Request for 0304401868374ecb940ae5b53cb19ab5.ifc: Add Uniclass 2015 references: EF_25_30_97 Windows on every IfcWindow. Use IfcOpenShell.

First a look at what the model holds.

```python
import ifcopenshell

model = ifcopenshell.open("0304401868374ecb940ae5b53cb19ab5.ifc")
print(model.schema)
print("classifications:", [c.Name for c in model.by_type("IfcClassification")])
for ifc_class in ("IfcDoor", "IfcRoof", "IfcStair", "IfcWall", "IfcWindow"):
    print(ifc_class, len(model.by_type(ifc_class)))
```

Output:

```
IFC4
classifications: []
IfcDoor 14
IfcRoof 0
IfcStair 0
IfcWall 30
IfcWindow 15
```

```python
import ifcopenshell
import ifcopenshell.api.classification

model = ifcopenshell.open("0304401868374ecb940ae5b53cb19ab5.ifc")

system = ifcopenshell.api.classification.add_classification(model, classification="Uniclass 2015")

codes = {
    "IfcWindow": ("EF_25_30_97", "Windows"),
}
for ifc_class, (code, name) in codes.items():
    products = model.by_type(ifc_class)
    ifcopenshell.api.classification.add_reference(
        model, products=products, classification=system, identification=code, name=name
    )
    print(code, len(products))

model.write("0304401868374ecb940ae5b53cb19ab5_v2.ifc")
```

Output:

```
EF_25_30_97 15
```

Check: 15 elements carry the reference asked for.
